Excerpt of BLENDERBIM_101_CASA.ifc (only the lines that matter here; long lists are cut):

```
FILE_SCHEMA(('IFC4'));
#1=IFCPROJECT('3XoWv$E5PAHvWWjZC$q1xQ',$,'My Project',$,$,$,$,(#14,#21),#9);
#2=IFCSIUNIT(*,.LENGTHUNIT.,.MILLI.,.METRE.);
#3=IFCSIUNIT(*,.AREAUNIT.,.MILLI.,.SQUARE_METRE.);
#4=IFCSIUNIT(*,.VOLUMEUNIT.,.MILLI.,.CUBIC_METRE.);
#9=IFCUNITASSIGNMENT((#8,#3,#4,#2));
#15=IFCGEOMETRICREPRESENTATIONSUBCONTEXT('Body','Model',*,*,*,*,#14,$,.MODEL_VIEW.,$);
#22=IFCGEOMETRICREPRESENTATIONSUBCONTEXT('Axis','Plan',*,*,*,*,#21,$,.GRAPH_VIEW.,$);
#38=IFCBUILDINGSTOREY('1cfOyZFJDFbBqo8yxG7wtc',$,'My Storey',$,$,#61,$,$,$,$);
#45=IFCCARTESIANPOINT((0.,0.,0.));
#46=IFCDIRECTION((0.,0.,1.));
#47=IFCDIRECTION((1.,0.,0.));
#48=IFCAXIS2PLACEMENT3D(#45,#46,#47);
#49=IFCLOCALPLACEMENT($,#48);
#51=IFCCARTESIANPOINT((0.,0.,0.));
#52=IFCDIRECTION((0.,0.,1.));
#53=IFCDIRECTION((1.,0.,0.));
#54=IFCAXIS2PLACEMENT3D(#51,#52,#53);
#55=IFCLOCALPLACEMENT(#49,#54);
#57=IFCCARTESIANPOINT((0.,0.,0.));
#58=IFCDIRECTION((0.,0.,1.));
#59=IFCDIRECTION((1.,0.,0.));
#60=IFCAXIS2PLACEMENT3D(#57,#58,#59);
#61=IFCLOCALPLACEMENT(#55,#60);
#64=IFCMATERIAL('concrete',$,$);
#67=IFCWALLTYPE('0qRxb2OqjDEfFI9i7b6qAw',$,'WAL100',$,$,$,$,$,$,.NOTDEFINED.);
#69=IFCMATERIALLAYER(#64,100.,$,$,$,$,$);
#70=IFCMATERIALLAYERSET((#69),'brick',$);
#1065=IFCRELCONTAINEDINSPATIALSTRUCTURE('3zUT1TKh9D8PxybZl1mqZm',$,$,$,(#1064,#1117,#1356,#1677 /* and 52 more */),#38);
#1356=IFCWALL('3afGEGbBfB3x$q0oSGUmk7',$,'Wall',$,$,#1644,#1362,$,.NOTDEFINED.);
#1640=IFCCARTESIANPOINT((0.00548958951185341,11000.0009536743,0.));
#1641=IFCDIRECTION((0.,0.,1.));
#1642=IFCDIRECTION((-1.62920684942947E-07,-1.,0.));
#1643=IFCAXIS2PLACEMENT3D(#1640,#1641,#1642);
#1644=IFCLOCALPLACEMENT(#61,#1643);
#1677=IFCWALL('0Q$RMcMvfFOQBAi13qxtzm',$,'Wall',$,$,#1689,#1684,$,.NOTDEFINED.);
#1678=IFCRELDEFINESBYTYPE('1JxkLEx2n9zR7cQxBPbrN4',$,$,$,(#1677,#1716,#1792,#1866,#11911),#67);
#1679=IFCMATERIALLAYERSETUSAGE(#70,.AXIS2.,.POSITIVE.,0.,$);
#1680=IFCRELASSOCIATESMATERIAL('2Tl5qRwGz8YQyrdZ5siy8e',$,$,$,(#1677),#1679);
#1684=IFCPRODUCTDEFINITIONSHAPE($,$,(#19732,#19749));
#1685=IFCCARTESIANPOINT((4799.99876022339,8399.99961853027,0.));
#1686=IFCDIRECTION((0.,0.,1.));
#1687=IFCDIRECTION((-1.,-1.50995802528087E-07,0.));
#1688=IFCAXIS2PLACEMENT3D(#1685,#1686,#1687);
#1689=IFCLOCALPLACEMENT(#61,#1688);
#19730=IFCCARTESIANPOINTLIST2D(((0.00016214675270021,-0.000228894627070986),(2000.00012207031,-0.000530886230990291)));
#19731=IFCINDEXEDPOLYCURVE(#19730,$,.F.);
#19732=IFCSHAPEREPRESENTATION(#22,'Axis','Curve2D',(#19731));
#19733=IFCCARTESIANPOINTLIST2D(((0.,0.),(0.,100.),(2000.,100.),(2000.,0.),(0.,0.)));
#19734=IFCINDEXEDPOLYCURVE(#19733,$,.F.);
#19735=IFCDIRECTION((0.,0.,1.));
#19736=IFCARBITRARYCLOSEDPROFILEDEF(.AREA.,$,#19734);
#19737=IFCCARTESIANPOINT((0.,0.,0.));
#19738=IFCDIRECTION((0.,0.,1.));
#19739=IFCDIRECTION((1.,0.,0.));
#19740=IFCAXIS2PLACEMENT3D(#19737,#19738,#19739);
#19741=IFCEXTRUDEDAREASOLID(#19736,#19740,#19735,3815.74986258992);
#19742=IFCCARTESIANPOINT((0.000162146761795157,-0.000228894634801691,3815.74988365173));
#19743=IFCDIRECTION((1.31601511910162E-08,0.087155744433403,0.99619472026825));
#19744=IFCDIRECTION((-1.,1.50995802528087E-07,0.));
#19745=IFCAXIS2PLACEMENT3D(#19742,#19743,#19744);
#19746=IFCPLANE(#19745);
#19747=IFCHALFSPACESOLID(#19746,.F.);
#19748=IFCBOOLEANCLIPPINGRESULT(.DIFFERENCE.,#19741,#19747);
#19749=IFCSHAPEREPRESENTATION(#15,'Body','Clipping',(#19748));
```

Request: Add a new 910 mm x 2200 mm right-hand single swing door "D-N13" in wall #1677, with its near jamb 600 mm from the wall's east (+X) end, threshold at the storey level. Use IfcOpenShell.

```python
import numpy as np
import ifcopenshell
import ifcopenshell.api.feature
import ifcopenshell.api.geometry
import ifcopenshell.api.root
import ifcopenshell.api.spatial
import ifcopenshell.geom
import ifcopenshell.util.element
import ifcopenshell.util.placement
import ifcopenshell.util.representation
import ifcopenshell.util.shape
import ifcopenshell.util.unit

model = ifcopenshell.open("BLENDERBIM_101_CASA.ifc")
unit_scale = ifcopenshell.util.unit.calculate_unit_scale(model)
settings = ifcopenshell.geom.settings()


def volume(element):
    """Net volume in cubic metres, openings subtracted."""
    shape = ifcopenshell.geom.create_shape(settings, element)
    return ifcopenshell.util.shape.get_volume(shape.geometry)


wall = model.by_id(1677)
storey = ifcopenshell.util.element.get_container(wall, ifc_class="IfcBuildingStorey")
context = ifcopenshell.util.representation.get_context(model, "Model", "Body", "MODEL_VIEW")
before = volume(wall)

width, height, from_end, sill = 0.91, 2.2, 0.6, 0.0  # metres

# The wall runs along its own X axis, and the end named is its -X end.
wall_shape = ifcopenshell.geom.create_shape(settings, wall)
x, y, z = ifcopenshell.util.shape.get_vertices(wall_shape.geometry).T
start = x.min() + from_end
face, thickness = float(y.min()), float(y.max() - y.min())
wall_matrix = ifcopenshell.util.placement.get_local_placement(wall.ObjectPlacement)
level = ifcopenshell.util.placement.get_local_placement(storey.ObjectPlacement)[2, 3]


def in_wall(x, y):
    """Placement at x, y metres in the wall's axes, at sill height."""
    matrix = wall_matrix.copy()
    matrix[:, 3] = wall_matrix @ np.array([x / unit_scale, y / unit_scale, 0.0, 1.0])
    matrix[2, 3] = level + sill / unit_scale
    return matrix


# Opening: a box that overshoots both wall faces by 50 mm.
opening = ifcopenshell.api.root.create_entity(model, ifc_class="IfcOpeningElement", predefined_type="OPENING")
box = ifcopenshell.api.geometry.add_wall_representation(
    model, context=context, length=width, height=height, thickness=thickness + 0.1
)
ifcopenshell.api.geometry.assign_representation(model, product=opening, representation=box)
ifcopenshell.api.geometry.edit_object_placement(model, product=opening, matrix=in_wall(start, face - 0.05), is_si=False)
ifcopenshell.api.feature.add_feature(model, feature=opening, element=wall)

door = ifcopenshell.api.root.create_entity(model, ifc_class="IfcDoor", name="D-N13", predefined_type="DOOR")
door.OverallWidth, door.OverallHeight = width / unit_scale, height / unit_scale
door.OperationType = "SINGLE_SWING_RIGHT"
body = ifcopenshell.api.geometry.add_door_representation(
    model,
    context=context,
    overall_width=door.OverallWidth,
    overall_height=door.OverallHeight,
    operation_type="SINGLE_SWING_RIGHT",
    lining_properties={"LiningDepth": thickness / unit_scale, "ThresholdDepth": thickness / unit_scale},
)
ifcopenshell.api.geometry.assign_representation(model, product=door, representation=body)
ifcopenshell.api.spatial.assign_container(model, products=[door], relating_structure=storey)
ifcopenshell.api.feature.add_filling(model, opening=opening, element=door)

# The lining spans the wall, so the door starts at the wall face.
ifcopenshell.api.geometry.edit_object_placement(model, product=door, matrix=in_wall(start, face), is_si=False)

after = volume(wall)

print(f"wall volume {before:.3f} -> {after:.3f} m3")

model.write("BLENDERBIM_101_CASA-out.ifc")
```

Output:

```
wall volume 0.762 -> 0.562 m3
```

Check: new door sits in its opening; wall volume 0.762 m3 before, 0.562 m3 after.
